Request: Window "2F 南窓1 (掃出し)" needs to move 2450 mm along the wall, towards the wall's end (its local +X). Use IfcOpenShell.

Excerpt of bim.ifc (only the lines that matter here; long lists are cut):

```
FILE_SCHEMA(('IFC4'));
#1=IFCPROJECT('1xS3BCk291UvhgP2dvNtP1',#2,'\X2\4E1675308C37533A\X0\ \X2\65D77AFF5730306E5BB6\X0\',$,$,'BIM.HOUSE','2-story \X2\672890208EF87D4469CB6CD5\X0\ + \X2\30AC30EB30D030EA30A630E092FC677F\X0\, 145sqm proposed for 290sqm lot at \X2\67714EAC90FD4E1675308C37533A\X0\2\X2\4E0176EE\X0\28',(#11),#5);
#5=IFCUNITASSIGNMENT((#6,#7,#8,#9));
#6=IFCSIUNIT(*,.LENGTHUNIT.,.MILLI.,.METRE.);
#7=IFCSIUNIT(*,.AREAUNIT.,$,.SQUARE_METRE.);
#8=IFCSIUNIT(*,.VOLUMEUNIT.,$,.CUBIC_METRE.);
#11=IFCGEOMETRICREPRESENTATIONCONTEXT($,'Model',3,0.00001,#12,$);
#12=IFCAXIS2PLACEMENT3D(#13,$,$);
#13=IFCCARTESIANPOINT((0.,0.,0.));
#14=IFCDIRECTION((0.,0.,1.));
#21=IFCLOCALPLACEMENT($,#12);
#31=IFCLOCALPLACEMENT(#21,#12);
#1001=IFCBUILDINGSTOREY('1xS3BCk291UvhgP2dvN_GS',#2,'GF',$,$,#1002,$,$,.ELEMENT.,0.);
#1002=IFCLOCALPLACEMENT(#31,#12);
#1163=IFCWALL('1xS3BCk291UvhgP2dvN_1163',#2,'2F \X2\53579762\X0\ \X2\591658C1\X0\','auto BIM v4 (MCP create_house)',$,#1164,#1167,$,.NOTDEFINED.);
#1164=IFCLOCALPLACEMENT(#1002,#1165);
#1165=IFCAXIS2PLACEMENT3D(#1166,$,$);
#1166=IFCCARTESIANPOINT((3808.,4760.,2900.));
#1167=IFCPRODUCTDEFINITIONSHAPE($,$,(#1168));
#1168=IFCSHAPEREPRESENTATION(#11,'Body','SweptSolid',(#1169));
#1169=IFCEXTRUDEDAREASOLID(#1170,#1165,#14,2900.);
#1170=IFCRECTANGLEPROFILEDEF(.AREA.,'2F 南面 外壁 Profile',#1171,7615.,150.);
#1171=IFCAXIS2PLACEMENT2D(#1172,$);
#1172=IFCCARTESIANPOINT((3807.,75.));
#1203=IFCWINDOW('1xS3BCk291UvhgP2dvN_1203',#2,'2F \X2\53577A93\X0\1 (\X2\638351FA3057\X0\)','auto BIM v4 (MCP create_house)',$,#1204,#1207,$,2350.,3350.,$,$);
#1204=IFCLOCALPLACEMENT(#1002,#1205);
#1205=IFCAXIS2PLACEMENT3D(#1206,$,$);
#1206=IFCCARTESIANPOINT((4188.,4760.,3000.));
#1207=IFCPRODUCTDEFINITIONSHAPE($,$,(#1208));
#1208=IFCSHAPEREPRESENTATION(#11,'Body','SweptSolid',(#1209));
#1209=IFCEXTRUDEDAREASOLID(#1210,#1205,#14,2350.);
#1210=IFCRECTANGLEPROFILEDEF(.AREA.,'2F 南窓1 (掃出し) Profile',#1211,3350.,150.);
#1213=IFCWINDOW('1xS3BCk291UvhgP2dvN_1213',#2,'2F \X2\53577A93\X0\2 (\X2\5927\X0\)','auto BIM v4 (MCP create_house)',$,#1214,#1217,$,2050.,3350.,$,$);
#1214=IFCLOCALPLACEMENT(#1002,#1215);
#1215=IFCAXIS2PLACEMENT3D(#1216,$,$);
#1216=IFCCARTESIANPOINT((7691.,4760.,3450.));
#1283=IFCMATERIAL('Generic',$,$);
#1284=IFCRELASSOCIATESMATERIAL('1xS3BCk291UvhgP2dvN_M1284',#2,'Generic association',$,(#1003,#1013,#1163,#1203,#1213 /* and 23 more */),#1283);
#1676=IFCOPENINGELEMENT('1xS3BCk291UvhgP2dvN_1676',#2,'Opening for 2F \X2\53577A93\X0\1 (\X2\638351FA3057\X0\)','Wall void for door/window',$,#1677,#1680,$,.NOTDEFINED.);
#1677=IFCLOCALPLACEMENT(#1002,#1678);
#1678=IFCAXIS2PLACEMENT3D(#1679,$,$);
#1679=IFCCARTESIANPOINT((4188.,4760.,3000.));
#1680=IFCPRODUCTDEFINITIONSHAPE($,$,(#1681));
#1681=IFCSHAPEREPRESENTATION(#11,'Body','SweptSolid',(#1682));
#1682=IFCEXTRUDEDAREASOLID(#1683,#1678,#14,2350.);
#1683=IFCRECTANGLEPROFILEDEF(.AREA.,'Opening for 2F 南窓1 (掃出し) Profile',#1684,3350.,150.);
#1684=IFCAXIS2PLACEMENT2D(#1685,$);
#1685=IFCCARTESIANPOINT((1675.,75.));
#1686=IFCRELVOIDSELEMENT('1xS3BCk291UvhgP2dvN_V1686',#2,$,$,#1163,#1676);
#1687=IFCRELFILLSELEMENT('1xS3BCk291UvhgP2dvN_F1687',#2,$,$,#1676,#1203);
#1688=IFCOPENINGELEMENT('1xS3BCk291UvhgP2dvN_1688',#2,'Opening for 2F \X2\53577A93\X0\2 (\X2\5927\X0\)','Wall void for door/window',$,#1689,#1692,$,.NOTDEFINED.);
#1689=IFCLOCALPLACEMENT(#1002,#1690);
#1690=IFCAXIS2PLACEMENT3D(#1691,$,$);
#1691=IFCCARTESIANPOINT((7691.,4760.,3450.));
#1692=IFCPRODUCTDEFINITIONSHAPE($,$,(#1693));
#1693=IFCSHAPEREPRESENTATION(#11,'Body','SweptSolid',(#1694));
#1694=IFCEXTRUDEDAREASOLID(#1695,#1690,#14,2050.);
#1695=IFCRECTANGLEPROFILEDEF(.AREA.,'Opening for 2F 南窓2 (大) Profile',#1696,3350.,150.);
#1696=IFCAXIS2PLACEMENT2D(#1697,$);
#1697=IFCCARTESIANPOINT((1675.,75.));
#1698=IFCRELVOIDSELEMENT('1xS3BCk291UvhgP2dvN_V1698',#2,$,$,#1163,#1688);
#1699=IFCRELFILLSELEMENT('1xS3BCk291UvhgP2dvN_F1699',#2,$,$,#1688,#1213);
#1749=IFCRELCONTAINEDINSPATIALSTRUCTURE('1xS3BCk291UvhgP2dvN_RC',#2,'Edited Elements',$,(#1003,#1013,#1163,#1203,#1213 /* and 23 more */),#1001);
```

```python
import ifcopenshell
import ifcopenshell.api.geometry
import ifcopenshell.util.placement

model = ifcopenshell.open("bim.ifc")

window = model.by_guid("1xS3BCk291UvhgP2dvN_1203")
opening = window.FillsVoids[0].RelatingOpeningElement
wall = opening.VoidsElements[0].RelatingBuildingElement

wall_matrix = ifcopenshell.util.placement.get_local_placement(wall.ObjectPlacement)
shift = wall_matrix[:3, 0] * 2450.0
before = ifcopenshell.util.placement.get_local_placement(window.ObjectPlacement)[:3, 3].copy()

# The window is not placed relative to its opening, so move both.
for product in (opening, window):
    matrix = ifcopenshell.util.placement.get_local_placement(product.ObjectPlacement)
    matrix[:3, 3] += shift
    ifcopenshell.api.geometry.edit_object_placement(model, product=product, matrix=matrix, is_si=False)

after = ifcopenshell.util.placement.get_local_placement(window.ObjectPlacement)[:3, 3]
print("window moved by", (after - before).round(3) + 0.0)

model.write("bim_v2.ifc")
```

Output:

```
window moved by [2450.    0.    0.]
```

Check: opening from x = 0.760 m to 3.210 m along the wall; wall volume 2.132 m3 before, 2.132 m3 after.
